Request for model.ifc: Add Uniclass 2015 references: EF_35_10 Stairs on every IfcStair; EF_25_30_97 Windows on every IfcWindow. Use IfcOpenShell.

First a look at what the model holds.

```python
import ifcopenshell

model = ifcopenshell.open("model.ifc")
print(model.schema)
print("classifications:", [c.Name for c in model.by_type("IfcClassification")])
for ifc_class in ("IfcDoor", "IfcRoof", "IfcStair", "IfcWall", "IfcWindow"):
    print(ifc_class, len(model.by_type(ifc_class)))
```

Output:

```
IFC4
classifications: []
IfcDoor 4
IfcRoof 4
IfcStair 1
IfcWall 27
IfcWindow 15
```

```python
import ifcopenshell
import ifcopenshell.api.classification

model = ifcopenshell.open("model.ifc")

system = ifcopenshell.api.classification.add_classification(model, classification="Uniclass 2015")

codes = {
    "IfcStair": ("EF_35_10", "Stairs"),
    "IfcWindow": ("EF_25_30_97", "Windows"),
}
for ifc_class, (code, name) in codes.items():
    products = model.by_type(ifc_class)
    ifcopenshell.api.classification.add_reference(
        model, products=products, classification=system, identification=code, name=name
    )
    print(code, len(products))

model.write("model_edited.ifc")
```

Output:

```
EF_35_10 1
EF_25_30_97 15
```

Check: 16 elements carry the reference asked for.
